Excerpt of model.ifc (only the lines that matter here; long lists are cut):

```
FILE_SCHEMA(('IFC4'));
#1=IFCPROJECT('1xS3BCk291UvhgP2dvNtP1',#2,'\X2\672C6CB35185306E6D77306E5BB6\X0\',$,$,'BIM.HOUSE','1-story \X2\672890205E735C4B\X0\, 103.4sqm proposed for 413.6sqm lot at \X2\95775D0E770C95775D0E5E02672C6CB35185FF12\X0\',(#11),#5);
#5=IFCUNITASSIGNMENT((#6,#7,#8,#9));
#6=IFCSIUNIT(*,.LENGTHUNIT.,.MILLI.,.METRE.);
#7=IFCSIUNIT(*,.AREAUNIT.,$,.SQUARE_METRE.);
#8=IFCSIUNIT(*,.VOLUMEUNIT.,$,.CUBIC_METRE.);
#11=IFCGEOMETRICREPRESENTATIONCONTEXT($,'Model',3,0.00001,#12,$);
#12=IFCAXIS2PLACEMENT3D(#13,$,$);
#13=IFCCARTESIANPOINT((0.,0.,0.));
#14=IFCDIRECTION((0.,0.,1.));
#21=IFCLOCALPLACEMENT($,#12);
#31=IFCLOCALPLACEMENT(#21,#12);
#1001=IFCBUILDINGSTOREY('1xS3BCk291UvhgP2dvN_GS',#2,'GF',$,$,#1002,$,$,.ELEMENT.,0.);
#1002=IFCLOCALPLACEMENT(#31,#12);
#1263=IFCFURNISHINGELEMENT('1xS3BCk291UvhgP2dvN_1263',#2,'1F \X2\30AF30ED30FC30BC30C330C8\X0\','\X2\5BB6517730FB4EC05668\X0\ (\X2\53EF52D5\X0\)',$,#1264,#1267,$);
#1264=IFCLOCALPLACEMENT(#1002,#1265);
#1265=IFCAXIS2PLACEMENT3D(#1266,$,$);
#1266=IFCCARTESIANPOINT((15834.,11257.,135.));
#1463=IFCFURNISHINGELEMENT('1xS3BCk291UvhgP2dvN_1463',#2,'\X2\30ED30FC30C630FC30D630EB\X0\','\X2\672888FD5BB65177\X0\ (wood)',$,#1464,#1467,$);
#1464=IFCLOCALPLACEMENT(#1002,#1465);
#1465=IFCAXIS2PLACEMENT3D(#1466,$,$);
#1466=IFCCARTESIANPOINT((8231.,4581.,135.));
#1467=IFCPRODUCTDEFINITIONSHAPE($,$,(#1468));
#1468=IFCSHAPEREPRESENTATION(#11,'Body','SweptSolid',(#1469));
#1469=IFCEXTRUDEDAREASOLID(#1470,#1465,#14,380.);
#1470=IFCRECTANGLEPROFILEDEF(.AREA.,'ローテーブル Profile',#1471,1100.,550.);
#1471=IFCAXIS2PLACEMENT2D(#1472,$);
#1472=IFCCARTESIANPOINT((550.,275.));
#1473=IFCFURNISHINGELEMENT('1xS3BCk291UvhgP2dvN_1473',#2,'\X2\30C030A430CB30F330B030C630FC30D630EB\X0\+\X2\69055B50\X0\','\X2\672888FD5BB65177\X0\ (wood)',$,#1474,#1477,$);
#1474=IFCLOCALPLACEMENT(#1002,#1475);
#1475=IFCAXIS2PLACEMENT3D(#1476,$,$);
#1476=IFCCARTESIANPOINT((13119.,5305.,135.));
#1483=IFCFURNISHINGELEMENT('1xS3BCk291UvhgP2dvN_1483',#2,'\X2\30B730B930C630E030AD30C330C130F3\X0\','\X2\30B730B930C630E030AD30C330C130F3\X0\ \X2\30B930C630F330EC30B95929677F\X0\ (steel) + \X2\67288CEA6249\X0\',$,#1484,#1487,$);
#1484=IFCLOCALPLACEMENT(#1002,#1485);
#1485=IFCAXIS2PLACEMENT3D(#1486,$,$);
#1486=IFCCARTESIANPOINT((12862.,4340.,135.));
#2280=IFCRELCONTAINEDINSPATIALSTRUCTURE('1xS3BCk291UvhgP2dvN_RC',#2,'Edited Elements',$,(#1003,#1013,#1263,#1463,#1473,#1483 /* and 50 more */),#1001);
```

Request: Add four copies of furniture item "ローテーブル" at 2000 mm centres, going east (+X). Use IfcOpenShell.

```python
import numpy as np
import ifcopenshell
import ifcopenshell.api.geometry
import ifcopenshell.api.root
import ifcopenshell.util.element
import ifcopenshell.util.placement

model = ifcopenshell.open("model.ifc")


def reuse_history(source, copy):
    """copy_class also copies each property set's owner history, people and application; keep the originals."""
    for rel in copy.IsDefinedBy:
        if rel.is_a("IfcRelDefinesByProperties") and (history := rel.RelatingPropertyDefinition.OwnerHistory):
            rel.RelatingPropertyDefinition.OwnerHistory = source.OwnerHistory
            ifcopenshell.util.element.remove_deep2(model, history)


source = model.by_id(1463)
base = ifcopenshell.util.placement.get_local_placement(source.ObjectPlacement)
step = np.array([1.0, 0.0, 0.0]) * 2000.0

for i in range(1, 5):
    copy = ifcopenshell.api.root.copy_class(model, product=source)
    copy.Representation = ifcopenshell.util.element.copy_deep(
        model, source.Representation, exclude=["IfcGeometricRepresentationContext", "IfcRepresentationMap"]
    )
    reuse_history(source, copy)
    matrix = base.copy()
    matrix[:3, 3] += i * step
    print("added at", matrix[:3, 3].round(3) + 0.0)
    ifcopenshell.api.geometry.edit_object_placement(model, product=copy, matrix=matrix, is_si=False)

model.write("model_v2.ifc")
```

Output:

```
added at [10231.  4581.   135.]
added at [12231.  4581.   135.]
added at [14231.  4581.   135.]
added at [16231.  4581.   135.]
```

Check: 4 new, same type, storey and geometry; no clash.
